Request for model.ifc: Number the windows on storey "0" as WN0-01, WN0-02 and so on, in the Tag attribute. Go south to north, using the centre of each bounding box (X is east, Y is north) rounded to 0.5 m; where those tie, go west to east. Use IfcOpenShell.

First a look at what the model holds.

```python
import ifcopenshell
import ifcopenshell.util.element
import ifcopenshell.util.placement

model = ifcopenshell.open("model.ifc")
print(model.schema)
storey = next(s for s in model.by_type("IfcBuildingStorey") if s.Name == "0")
windows = [e for e in ifcopenshell.util.element.get_decomposition(storey) if e.is_a("IfcWindow")]
for e in sorted(windows, key=lambda e: e.id()):
    origin = ifcopenshell.util.placement.get_local_placement(e.ObjectPlacement)[:3, 3]
    print(e.id(), e.Tag, e.Name, origin.round(2) + 0.0, sep=" | ")
```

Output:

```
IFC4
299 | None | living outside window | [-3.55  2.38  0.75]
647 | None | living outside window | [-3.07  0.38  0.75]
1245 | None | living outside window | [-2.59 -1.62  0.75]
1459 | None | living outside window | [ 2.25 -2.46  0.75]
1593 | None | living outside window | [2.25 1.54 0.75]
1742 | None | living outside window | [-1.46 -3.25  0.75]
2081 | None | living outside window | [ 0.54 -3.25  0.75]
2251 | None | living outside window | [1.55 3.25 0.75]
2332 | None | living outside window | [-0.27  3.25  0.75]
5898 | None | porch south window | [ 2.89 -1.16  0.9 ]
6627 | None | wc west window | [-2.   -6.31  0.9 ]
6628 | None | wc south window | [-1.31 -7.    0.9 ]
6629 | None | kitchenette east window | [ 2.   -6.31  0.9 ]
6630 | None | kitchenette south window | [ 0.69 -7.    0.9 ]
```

```python
import ifcopenshell
import ifcopenshell.geom
import ifcopenshell.util.element
import ifcopenshell.util.shape

model = ifcopenshell.open("model.ifc")
settings = ifcopenshell.geom.settings()
settings.set("use-world-coords", True)


def centre(element):
    shape = ifcopenshell.geom.create_shape(settings, element)
    return ifcopenshell.util.shape.get_bbox_centroid(shape.geometry)


storey = next(s for s in model.by_type("IfcBuildingStorey") if s.Name == "0")
windows = [e for e in ifcopenshell.util.element.get_decomposition(storey) if e.is_a("IfcWindow")]

# Insertion points can sit at a corner or the storey origin, so sort by the geometry (in metres).
centres = {e: centre(e) for e in windows}
windows.sort(key=lambda e: (round(centres[e][1] / 0.5), centres[e][0]))

for i, e in enumerate(windows, start=1):
    number = f"WN0-{i:02d}"
    e.Tag = number
    print(e.id(), number)

model.write("model-out.ifc")
```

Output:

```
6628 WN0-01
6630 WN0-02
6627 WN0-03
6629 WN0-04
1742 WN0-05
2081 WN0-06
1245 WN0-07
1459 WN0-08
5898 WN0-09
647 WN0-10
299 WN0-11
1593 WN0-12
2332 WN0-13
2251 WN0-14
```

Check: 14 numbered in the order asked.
